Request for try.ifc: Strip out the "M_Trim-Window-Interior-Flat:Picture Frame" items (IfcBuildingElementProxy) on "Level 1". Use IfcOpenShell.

First a look at what the model holds.

```python
import ifcopenshell
import ifcopenshell.util.element

model = ifcopenshell.open("try.ifc")
print(model.schema)
storey = next(s for s in model.by_type("IfcBuildingStorey") if s.Name == "Level 1")
proxies = [e for e in ifcopenshell.util.element.get_decomposition(storey) if e.is_a("IfcBuildingElementProxy")]
seen = {}
for e in proxies:
    element_type = ifcopenshell.util.element.get_type(e)
    name = element_type.Name if element_type not in (None, e) else None
    seen[name] = seen.get(name, 0) + 1
for name, count in sorted(seen.items(), key=str):
    print(count, "x", name)
```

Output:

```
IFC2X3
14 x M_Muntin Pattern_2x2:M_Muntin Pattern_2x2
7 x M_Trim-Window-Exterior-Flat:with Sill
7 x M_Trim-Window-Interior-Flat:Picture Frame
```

```python
import ifcopenshell
import ifcopenshell.api.root
import ifcopenshell.util.element

model = ifcopenshell.open("try.ifc")

storey = next(s for s in model.by_type("IfcBuildingStorey") if s.Name == "Level 1")
proxies = [e for e in ifcopenshell.util.element.get_decomposition(storey) if e.is_a("IfcBuildingElementProxy")]
targets = [e for e in proxies if (t := ifcopenshell.util.element.get_type(e)) not in (None, e) and t.Name == "M_Trim-Window-Interior-Flat:Picture Frame"]

for e in targets:
    ifcopenshell.api.root.remove_product(model, product=e)
print(len(targets), "removed")

model.write("try_v2.ifc")
```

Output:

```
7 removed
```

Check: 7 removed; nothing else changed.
